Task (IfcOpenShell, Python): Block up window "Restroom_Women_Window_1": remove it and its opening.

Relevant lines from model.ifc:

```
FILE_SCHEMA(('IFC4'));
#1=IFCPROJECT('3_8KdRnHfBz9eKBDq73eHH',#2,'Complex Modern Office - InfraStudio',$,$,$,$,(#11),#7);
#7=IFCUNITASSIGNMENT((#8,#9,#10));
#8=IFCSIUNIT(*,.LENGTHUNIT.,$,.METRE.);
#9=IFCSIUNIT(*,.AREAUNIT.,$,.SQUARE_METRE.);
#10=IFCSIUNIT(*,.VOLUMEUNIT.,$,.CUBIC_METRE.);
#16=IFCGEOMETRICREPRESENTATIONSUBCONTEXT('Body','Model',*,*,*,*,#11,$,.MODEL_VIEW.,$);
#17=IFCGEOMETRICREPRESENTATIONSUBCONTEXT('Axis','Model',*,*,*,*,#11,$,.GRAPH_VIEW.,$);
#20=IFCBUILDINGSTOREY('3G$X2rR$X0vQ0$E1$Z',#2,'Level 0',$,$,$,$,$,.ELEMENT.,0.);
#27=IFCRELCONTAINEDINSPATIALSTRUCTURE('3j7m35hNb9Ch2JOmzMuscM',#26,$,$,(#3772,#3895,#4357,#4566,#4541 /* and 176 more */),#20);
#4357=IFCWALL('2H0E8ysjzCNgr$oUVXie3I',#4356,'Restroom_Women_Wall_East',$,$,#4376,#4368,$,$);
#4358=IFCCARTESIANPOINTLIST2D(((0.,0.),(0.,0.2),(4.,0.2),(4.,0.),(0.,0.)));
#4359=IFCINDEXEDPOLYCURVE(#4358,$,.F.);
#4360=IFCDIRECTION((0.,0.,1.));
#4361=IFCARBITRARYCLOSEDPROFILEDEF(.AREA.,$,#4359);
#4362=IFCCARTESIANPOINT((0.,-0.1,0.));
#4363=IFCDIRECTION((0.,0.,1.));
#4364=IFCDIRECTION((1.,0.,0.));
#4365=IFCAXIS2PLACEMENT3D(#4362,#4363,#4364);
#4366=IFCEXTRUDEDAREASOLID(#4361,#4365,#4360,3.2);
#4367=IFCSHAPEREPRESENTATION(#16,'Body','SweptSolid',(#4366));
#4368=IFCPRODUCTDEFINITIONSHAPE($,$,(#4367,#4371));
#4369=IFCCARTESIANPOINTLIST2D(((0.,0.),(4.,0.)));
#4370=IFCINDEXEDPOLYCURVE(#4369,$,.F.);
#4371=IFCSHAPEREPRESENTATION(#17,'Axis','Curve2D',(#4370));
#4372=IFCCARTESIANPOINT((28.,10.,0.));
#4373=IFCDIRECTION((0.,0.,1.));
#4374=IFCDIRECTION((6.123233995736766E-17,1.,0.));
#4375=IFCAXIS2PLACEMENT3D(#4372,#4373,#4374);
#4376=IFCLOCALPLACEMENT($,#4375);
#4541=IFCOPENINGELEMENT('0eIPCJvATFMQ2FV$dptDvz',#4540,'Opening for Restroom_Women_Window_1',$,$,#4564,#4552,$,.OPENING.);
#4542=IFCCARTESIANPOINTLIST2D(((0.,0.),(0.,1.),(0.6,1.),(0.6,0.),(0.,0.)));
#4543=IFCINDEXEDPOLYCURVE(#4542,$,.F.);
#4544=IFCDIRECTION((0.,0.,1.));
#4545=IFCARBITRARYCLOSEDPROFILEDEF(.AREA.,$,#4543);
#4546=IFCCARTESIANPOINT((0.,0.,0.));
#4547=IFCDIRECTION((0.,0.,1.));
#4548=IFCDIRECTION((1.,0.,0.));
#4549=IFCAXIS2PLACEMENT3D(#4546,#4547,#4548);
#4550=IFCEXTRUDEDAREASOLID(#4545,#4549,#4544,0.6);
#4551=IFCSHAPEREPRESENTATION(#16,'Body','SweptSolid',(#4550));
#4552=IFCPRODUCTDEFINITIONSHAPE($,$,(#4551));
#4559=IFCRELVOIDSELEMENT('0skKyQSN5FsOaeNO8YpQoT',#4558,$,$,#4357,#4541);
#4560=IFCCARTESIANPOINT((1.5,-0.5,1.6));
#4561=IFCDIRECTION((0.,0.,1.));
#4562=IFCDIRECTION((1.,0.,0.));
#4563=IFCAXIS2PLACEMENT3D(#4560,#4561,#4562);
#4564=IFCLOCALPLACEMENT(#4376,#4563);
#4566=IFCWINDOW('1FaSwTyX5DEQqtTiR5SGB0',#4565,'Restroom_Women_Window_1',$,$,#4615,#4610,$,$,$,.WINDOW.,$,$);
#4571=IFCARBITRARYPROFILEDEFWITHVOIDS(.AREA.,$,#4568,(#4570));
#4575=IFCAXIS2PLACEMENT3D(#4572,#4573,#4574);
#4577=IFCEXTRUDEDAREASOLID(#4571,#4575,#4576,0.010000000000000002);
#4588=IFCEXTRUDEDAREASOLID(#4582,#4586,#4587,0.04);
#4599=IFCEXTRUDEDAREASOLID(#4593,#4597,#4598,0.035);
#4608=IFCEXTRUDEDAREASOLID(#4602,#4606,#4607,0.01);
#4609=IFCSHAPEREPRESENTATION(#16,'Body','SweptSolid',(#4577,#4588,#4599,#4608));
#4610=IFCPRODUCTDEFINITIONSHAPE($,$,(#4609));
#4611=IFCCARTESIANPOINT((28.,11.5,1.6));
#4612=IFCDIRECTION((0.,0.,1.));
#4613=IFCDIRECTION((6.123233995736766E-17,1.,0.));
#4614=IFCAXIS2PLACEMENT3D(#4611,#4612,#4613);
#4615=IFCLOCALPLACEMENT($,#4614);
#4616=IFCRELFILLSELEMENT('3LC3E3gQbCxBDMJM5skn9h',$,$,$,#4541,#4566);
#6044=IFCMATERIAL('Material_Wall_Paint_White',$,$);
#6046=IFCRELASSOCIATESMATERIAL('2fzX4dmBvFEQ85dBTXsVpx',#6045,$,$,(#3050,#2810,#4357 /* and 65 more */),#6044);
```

```python
import ifcopenshell
import ifcopenshell.api.feature
import ifcopenshell.api.root
import ifcopenshell.geom
import ifcopenshell.util.shape

model = ifcopenshell.open("model.ifc")
settings = ifcopenshell.geom.settings()


def volume(element):
    """Net volume in cubic metres, openings subtracted."""
    shape = ifcopenshell.geom.create_shape(settings, element)
    return ifcopenshell.util.shape.get_volume(shape.geometry)


window = model.by_id(4566)
opening = window.FillsVoids[0].RelatingOpeningElement
wall = opening.VoidsElements[0].RelatingBuildingElement
before = volume(wall)

ifcopenshell.api.root.remove_product(model, product=window)
ifcopenshell.api.feature.remove_feature(model, feature=opening)

after = volume(wall)

print(f"wall volume {before:.3f} -> {after:.3f} m3")

model.write("model_updated.ifc")
```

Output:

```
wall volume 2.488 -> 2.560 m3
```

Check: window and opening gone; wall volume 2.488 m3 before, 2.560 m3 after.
